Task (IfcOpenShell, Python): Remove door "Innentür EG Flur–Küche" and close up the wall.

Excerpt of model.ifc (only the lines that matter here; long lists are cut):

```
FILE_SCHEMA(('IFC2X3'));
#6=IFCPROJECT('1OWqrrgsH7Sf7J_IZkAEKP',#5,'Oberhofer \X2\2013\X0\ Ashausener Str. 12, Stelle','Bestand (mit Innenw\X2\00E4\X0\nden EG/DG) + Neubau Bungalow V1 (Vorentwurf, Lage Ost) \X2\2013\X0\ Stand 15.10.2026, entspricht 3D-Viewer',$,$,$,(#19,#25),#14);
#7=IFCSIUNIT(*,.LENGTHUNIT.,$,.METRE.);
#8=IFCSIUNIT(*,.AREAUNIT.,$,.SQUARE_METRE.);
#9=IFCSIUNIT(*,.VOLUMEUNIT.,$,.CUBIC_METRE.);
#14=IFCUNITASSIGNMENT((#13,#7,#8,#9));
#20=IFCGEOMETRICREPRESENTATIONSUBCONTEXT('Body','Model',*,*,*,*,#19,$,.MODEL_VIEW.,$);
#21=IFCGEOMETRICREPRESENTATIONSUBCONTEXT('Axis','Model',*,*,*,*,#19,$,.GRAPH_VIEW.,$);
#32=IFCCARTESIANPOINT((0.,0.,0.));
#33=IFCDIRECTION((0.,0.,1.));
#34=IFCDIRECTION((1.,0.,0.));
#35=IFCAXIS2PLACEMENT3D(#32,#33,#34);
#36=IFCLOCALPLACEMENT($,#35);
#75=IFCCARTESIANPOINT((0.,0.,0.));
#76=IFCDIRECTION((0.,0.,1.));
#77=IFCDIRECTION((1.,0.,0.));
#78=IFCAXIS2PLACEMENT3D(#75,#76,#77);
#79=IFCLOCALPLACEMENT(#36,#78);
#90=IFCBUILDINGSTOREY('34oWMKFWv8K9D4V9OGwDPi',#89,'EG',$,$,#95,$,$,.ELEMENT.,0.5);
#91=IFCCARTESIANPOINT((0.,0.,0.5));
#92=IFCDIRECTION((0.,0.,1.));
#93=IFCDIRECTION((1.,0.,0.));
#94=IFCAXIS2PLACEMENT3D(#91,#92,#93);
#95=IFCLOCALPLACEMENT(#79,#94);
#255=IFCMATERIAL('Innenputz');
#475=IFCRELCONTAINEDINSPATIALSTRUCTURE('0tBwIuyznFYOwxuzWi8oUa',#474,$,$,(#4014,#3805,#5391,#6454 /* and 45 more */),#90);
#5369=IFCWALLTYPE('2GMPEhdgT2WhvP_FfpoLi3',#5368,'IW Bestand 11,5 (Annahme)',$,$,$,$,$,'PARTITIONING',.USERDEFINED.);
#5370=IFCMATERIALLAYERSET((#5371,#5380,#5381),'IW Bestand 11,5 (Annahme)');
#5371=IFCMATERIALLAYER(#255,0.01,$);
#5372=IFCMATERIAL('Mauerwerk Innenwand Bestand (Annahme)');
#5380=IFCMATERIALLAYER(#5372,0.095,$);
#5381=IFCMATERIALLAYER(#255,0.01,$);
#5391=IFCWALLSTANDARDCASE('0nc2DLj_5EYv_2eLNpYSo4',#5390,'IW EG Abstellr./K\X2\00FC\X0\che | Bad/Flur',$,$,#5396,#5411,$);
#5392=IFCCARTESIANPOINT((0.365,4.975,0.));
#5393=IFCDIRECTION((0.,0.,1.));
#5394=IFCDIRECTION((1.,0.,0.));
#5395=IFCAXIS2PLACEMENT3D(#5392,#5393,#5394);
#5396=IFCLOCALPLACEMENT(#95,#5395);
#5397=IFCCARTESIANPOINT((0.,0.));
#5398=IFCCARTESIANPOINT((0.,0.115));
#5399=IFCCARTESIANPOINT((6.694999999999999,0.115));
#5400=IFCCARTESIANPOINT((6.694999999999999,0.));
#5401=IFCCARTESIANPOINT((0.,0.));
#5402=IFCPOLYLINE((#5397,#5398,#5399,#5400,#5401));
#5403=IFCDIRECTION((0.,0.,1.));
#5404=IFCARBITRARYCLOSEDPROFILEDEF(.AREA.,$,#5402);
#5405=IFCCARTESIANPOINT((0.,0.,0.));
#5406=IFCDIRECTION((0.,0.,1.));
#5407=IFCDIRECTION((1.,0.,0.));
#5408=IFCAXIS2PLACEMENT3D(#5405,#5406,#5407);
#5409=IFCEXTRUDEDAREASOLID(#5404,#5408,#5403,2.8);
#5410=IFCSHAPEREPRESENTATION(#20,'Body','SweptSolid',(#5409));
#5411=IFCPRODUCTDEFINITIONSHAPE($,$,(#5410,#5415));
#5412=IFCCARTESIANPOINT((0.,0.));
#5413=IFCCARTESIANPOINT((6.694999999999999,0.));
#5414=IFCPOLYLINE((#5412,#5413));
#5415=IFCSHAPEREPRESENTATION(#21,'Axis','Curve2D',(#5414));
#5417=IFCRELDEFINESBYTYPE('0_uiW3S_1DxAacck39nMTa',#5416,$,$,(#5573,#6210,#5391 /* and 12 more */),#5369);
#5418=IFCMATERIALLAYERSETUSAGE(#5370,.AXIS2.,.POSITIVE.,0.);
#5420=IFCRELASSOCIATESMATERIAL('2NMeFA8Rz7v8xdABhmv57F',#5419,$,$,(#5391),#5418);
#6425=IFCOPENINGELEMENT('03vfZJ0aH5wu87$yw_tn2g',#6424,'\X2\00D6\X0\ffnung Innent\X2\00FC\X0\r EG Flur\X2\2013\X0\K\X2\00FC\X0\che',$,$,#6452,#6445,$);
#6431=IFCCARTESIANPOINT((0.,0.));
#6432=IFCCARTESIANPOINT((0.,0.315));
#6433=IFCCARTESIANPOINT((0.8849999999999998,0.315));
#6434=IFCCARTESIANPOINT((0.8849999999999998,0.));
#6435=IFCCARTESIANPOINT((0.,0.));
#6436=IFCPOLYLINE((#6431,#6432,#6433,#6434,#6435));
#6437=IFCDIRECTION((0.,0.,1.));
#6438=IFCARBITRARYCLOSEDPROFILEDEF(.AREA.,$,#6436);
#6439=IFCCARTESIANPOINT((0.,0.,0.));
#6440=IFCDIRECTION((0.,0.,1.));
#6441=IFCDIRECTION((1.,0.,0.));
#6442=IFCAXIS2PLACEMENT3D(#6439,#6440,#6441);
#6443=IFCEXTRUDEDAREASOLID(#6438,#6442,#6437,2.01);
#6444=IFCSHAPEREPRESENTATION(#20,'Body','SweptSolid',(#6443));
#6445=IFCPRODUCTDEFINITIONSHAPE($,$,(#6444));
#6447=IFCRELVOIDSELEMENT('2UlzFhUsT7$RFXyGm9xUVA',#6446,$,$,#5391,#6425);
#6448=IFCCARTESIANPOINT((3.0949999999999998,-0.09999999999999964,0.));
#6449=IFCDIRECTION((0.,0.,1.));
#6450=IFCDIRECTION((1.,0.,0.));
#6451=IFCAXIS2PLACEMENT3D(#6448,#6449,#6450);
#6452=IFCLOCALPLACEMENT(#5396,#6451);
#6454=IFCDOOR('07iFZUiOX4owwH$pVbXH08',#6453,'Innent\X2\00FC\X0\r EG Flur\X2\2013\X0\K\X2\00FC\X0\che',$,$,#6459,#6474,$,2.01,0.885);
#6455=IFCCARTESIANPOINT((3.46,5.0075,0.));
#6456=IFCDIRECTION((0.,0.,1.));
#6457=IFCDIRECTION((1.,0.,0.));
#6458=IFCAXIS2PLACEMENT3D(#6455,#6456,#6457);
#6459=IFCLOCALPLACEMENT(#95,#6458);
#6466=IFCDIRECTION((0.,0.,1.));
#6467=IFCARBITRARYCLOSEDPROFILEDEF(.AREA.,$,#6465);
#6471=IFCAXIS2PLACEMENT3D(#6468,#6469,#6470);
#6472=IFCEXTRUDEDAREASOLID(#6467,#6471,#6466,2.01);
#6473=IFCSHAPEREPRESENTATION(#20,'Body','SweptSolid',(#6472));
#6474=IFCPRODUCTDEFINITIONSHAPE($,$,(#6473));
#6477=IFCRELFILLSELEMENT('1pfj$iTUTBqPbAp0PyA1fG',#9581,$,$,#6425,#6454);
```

```python
import ifcopenshell
import ifcopenshell.api.feature
import ifcopenshell.api.root
import ifcopenshell.geom
import ifcopenshell.util.shape

model = ifcopenshell.open("model.ifc")
settings = ifcopenshell.geom.settings()


def volume(element):
    """Net volume in cubic metres, openings subtracted."""
    shape = ifcopenshell.geom.create_shape(settings, element)
    return ifcopenshell.util.shape.get_volume(shape.geometry)


door = model.by_guid("07iFZUiOX4owwH$pVbXH08")
opening = door.FillsVoids[0].RelatingOpeningElement
wall = opening.VoidsElements[0].RelatingBuildingElement
before = volume(wall)

ifcopenshell.api.root.remove_product(model, product=door)
ifcopenshell.api.feature.remove_feature(model, feature=opening)

after = volume(wall)

print(f"wall volume {before:.3f} -> {after:.3f} m3")

model.write("model-out.ifc")
```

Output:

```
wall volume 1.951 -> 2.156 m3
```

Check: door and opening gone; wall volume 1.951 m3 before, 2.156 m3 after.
